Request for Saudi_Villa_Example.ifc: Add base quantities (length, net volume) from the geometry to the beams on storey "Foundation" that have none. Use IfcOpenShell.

First a look at what the model holds.

```python
import ifcopenshell
import ifcopenshell.util.element
import ifcopenshell.util.unit

model = ifcopenshell.open("Saudi_Villa_Example.ifc")
print(model.schema)
for unit_type in ("LENGTHUNIT", "AREAUNIT", "VOLUMEUNIT"):
    print(unit_type, ifcopenshell.util.unit.calculate_unit_scale(model, unit_type))
storey = next(s for s in model.by_type("IfcBuildingStorey") if s.Name == "Foundation")
beams = [e for e in ifcopenshell.util.element.get_decomposition(storey) if e.is_a("IfcBeam")]
for e in sorted(beams, key=lambda e: e.id()):
    print(e.id(), e.is_a(), e.Name, list(ifcopenshell.util.element.get_psets(e, qtos_only=True)), sep=" | ")
```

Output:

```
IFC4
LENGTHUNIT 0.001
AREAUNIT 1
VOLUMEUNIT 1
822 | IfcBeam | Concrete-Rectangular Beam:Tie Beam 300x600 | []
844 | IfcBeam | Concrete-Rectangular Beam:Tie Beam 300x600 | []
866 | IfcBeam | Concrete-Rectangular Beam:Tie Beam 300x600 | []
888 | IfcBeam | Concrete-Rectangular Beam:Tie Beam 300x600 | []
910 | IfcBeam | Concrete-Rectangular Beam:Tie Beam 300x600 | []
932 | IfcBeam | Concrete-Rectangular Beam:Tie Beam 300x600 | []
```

```python
import ifcopenshell
import ifcopenshell.api.pset
import ifcopenshell.geom
import ifcopenshell.util.element
import ifcopenshell.util.shape
import ifcopenshell.util.unit

model = ifcopenshell.open("Saudi_Villa_Example.ifc")
unit_scale = ifcopenshell.util.unit.calculate_unit_scale(model)
volume_scale = ifcopenshell.util.unit.calculate_unit_scale(model, "VOLUMEUNIT")
settings = ifcopenshell.geom.settings()

storey = next(s for s in model.by_type("IfcBuildingStorey") if s.Name == "Foundation")
beams = [e for e in ifcopenshell.util.element.get_decomposition(storey) if e.is_a("IfcBeam")]

for e in sorted(beams, key=lambda e: e.id()):
    if ifcopenshell.util.element.get_psets(e, qtos_only=True, should_inherit=False):
        continue
    # Geometry comes back in metres, in the element's own axes.
    shape = ifcopenshell.geom.create_shape(settings, e)
    values = {
        "Length": ifcopenshell.util.shape.get_max_xyz(shape.geometry) / unit_scale,
        "NetVolume": ifcopenshell.util.shape.get_volume(shape.geometry) / volume_scale,
    }
    qto = ifcopenshell.api.pset.add_qto(model, product=e, name="Qto_BeamBaseQuantities")
    ifcopenshell.api.pset.edit_qto(model, qto=qto, properties=values)
    print(e.id(), {k: round(v, 3) for k, v in values.items()})

model.write("Saudi_Villa_Example_updated.ifc")
```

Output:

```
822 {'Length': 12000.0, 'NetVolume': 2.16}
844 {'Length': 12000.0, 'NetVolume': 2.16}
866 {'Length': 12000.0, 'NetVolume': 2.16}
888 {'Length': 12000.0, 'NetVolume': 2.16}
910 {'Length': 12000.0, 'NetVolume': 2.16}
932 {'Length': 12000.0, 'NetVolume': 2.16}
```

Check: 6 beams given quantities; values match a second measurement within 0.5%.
